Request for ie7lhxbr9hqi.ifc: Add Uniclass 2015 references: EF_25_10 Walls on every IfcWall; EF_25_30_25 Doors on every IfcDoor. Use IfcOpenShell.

First a look at what the model holds.

```python
import ifcopenshell

model = ifcopenshell.open("ie7lhxbr9hqi.ifc")
print(model.schema)
print("classifications:", [c.Name for c in model.by_type("IfcClassification")])
for ifc_class in ("IfcDoor", "IfcRoof", "IfcStair", "IfcWall", "IfcWindow"):
    print(ifc_class, len(model.by_type(ifc_class)))
```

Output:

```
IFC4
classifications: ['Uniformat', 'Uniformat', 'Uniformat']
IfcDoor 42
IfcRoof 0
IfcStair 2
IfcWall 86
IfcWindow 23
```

```python
import ifcopenshell
import ifcopenshell.api.classification

model = ifcopenshell.open("ie7lhxbr9hqi.ifc")

system = ifcopenshell.api.classification.add_classification(model, classification="Uniclass 2015")

codes = {
    "IfcWall": ("EF_25_10", "Walls"),
    "IfcDoor": ("EF_25_30_25", "Doors"),
}
for ifc_class, (code, name) in codes.items():
    products = model.by_type(ifc_class)
    ifcopenshell.api.classification.add_reference(
        model, products=products, classification=system, identification=code, name=name
    )
    print(code, len(products))

model.write("ie7lhxbr9hqi_v2.ifc")
```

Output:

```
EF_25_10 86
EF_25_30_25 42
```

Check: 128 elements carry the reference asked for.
